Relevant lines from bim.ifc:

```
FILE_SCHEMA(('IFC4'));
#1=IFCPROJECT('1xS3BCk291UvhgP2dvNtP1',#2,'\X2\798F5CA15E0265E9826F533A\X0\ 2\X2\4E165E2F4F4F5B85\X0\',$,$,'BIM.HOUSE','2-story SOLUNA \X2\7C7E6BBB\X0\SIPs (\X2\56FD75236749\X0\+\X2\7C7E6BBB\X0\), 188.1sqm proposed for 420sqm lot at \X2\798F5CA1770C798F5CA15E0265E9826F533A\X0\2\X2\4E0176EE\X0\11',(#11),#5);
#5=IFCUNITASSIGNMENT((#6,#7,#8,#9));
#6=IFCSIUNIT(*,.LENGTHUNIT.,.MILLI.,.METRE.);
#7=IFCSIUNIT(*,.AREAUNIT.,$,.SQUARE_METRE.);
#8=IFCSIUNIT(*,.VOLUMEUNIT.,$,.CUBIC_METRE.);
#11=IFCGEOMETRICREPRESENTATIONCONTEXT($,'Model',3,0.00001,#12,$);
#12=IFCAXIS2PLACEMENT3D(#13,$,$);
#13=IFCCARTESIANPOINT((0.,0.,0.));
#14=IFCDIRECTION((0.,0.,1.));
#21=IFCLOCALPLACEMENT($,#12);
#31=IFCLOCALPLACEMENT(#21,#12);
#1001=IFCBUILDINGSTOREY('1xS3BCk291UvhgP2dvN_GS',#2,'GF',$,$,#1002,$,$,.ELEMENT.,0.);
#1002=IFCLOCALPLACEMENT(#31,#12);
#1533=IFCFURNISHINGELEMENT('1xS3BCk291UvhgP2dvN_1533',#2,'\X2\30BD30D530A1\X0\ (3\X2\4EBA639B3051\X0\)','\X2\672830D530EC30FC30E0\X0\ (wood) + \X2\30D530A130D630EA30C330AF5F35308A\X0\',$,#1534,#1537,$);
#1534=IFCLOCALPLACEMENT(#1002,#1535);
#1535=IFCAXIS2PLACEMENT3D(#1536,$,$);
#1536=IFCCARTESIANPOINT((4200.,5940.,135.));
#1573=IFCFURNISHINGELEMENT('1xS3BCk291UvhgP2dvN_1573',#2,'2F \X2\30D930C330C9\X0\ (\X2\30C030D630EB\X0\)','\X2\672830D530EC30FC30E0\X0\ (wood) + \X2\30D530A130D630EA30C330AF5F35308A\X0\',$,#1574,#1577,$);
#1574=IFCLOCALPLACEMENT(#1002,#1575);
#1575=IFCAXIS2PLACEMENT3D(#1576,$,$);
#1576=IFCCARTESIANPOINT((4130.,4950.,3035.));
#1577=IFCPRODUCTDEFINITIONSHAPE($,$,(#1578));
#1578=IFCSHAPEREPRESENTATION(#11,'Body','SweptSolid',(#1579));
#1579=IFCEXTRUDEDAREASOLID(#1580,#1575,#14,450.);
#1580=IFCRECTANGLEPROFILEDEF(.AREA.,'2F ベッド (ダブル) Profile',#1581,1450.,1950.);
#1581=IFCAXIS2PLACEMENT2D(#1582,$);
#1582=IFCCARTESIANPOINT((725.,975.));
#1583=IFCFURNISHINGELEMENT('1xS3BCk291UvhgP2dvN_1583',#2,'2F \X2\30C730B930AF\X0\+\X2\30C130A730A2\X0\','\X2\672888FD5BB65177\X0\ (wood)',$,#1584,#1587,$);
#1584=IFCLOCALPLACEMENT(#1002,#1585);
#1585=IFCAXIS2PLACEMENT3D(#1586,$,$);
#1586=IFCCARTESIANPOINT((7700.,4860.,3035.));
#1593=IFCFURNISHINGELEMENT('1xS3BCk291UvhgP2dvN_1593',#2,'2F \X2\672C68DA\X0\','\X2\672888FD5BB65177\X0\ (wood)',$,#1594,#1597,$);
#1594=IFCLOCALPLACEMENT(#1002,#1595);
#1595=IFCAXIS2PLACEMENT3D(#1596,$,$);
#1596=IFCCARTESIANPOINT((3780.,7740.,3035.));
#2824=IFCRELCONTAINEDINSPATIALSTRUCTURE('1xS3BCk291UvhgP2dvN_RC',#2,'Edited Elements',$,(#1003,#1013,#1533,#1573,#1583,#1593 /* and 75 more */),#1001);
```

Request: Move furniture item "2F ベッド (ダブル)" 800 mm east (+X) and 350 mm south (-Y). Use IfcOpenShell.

```python
import ifcopenshell
import ifcopenshell.api.geometry
import ifcopenshell.util.placement

model = ifcopenshell.open("bim.ifc")

item = model.by_id(1573)
matrix = ifcopenshell.util.placement.get_local_placement(item.ObjectPlacement)
matrix[0, 3] += 800.0
matrix[1, 3] -= 350.0
ifcopenshell.api.geometry.edit_object_placement(model, product=item, matrix=matrix, is_si=False)

print(ifcopenshell.util.placement.get_local_placement(item.ObjectPlacement).round(3) + 0.0)

model.write("bim_edited.ifc")
```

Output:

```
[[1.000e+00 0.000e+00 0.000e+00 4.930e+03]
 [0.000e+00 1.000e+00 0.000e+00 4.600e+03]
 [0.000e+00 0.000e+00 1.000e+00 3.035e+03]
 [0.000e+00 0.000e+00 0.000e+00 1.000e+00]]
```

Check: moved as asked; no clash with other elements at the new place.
